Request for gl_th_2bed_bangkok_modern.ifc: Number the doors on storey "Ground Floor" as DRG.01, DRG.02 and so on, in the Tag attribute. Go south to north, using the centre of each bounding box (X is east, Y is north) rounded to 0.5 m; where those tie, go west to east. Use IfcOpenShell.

First a look at what the model holds.

```python
import ifcopenshell
import ifcopenshell.util.element
import ifcopenshell.util.placement

model = ifcopenshell.open("gl_th_2bed_bangkok_modern.ifc")
print(model.schema)
storey = next(s for s in model.by_type("IfcBuildingStorey") if s.Name == "Ground Floor")
doors = [e for e in ifcopenshell.util.element.get_decomposition(storey) if e.is_a("IfcDoor")]
for e in sorted(doors, key=lambda e: e.id()):
    origin = ifcopenshell.util.placement.get_local_placement(e.ObjectPlacement)[:3, 3]
    print(e.id(), e.Tag, e.Name, origin.round(2) + 0.0, sep=" | ")
```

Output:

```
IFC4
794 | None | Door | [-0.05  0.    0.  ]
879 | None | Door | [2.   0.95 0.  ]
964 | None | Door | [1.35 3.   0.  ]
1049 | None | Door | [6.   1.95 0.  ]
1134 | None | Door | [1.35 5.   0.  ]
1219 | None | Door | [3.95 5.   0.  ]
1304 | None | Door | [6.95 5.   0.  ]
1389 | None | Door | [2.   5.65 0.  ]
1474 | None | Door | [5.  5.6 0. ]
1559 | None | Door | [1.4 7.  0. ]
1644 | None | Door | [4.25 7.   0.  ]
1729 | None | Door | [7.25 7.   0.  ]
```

```python
import ifcopenshell
import ifcopenshell.geom
import ifcopenshell.util.element
import ifcopenshell.util.shape

model = ifcopenshell.open("gl_th_2bed_bangkok_modern.ifc")
settings = ifcopenshell.geom.settings()
settings.set("use-world-coords", True)


def centre(element):
    shape = ifcopenshell.geom.create_shape(settings, element)
    return ifcopenshell.util.shape.get_bbox_centroid(shape.geometry)


storey = next(s for s in model.by_type("IfcBuildingStorey") if s.Name == "Ground Floor")
doors = [e for e in ifcopenshell.util.element.get_decomposition(storey) if e.is_a("IfcDoor")]

# Insertion points can sit at a corner or the storey origin, so sort by the geometry (in metres).
centres = {e: centre(e) for e in doors}
doors.sort(key=lambda e: (round(centres[e][1] / 0.5), centres[e][0]))

for i, e in enumerate(doors, start=1):
    number = f"DRG.{i:02d}"
    e.Tag = number
    print(e.id(), number)

model.write("gl_th_2bed_bangkok_modern_updated.ifc")
```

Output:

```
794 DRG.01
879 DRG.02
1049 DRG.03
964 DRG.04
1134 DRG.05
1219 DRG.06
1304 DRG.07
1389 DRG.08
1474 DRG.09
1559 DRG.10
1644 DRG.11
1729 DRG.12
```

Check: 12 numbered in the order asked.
